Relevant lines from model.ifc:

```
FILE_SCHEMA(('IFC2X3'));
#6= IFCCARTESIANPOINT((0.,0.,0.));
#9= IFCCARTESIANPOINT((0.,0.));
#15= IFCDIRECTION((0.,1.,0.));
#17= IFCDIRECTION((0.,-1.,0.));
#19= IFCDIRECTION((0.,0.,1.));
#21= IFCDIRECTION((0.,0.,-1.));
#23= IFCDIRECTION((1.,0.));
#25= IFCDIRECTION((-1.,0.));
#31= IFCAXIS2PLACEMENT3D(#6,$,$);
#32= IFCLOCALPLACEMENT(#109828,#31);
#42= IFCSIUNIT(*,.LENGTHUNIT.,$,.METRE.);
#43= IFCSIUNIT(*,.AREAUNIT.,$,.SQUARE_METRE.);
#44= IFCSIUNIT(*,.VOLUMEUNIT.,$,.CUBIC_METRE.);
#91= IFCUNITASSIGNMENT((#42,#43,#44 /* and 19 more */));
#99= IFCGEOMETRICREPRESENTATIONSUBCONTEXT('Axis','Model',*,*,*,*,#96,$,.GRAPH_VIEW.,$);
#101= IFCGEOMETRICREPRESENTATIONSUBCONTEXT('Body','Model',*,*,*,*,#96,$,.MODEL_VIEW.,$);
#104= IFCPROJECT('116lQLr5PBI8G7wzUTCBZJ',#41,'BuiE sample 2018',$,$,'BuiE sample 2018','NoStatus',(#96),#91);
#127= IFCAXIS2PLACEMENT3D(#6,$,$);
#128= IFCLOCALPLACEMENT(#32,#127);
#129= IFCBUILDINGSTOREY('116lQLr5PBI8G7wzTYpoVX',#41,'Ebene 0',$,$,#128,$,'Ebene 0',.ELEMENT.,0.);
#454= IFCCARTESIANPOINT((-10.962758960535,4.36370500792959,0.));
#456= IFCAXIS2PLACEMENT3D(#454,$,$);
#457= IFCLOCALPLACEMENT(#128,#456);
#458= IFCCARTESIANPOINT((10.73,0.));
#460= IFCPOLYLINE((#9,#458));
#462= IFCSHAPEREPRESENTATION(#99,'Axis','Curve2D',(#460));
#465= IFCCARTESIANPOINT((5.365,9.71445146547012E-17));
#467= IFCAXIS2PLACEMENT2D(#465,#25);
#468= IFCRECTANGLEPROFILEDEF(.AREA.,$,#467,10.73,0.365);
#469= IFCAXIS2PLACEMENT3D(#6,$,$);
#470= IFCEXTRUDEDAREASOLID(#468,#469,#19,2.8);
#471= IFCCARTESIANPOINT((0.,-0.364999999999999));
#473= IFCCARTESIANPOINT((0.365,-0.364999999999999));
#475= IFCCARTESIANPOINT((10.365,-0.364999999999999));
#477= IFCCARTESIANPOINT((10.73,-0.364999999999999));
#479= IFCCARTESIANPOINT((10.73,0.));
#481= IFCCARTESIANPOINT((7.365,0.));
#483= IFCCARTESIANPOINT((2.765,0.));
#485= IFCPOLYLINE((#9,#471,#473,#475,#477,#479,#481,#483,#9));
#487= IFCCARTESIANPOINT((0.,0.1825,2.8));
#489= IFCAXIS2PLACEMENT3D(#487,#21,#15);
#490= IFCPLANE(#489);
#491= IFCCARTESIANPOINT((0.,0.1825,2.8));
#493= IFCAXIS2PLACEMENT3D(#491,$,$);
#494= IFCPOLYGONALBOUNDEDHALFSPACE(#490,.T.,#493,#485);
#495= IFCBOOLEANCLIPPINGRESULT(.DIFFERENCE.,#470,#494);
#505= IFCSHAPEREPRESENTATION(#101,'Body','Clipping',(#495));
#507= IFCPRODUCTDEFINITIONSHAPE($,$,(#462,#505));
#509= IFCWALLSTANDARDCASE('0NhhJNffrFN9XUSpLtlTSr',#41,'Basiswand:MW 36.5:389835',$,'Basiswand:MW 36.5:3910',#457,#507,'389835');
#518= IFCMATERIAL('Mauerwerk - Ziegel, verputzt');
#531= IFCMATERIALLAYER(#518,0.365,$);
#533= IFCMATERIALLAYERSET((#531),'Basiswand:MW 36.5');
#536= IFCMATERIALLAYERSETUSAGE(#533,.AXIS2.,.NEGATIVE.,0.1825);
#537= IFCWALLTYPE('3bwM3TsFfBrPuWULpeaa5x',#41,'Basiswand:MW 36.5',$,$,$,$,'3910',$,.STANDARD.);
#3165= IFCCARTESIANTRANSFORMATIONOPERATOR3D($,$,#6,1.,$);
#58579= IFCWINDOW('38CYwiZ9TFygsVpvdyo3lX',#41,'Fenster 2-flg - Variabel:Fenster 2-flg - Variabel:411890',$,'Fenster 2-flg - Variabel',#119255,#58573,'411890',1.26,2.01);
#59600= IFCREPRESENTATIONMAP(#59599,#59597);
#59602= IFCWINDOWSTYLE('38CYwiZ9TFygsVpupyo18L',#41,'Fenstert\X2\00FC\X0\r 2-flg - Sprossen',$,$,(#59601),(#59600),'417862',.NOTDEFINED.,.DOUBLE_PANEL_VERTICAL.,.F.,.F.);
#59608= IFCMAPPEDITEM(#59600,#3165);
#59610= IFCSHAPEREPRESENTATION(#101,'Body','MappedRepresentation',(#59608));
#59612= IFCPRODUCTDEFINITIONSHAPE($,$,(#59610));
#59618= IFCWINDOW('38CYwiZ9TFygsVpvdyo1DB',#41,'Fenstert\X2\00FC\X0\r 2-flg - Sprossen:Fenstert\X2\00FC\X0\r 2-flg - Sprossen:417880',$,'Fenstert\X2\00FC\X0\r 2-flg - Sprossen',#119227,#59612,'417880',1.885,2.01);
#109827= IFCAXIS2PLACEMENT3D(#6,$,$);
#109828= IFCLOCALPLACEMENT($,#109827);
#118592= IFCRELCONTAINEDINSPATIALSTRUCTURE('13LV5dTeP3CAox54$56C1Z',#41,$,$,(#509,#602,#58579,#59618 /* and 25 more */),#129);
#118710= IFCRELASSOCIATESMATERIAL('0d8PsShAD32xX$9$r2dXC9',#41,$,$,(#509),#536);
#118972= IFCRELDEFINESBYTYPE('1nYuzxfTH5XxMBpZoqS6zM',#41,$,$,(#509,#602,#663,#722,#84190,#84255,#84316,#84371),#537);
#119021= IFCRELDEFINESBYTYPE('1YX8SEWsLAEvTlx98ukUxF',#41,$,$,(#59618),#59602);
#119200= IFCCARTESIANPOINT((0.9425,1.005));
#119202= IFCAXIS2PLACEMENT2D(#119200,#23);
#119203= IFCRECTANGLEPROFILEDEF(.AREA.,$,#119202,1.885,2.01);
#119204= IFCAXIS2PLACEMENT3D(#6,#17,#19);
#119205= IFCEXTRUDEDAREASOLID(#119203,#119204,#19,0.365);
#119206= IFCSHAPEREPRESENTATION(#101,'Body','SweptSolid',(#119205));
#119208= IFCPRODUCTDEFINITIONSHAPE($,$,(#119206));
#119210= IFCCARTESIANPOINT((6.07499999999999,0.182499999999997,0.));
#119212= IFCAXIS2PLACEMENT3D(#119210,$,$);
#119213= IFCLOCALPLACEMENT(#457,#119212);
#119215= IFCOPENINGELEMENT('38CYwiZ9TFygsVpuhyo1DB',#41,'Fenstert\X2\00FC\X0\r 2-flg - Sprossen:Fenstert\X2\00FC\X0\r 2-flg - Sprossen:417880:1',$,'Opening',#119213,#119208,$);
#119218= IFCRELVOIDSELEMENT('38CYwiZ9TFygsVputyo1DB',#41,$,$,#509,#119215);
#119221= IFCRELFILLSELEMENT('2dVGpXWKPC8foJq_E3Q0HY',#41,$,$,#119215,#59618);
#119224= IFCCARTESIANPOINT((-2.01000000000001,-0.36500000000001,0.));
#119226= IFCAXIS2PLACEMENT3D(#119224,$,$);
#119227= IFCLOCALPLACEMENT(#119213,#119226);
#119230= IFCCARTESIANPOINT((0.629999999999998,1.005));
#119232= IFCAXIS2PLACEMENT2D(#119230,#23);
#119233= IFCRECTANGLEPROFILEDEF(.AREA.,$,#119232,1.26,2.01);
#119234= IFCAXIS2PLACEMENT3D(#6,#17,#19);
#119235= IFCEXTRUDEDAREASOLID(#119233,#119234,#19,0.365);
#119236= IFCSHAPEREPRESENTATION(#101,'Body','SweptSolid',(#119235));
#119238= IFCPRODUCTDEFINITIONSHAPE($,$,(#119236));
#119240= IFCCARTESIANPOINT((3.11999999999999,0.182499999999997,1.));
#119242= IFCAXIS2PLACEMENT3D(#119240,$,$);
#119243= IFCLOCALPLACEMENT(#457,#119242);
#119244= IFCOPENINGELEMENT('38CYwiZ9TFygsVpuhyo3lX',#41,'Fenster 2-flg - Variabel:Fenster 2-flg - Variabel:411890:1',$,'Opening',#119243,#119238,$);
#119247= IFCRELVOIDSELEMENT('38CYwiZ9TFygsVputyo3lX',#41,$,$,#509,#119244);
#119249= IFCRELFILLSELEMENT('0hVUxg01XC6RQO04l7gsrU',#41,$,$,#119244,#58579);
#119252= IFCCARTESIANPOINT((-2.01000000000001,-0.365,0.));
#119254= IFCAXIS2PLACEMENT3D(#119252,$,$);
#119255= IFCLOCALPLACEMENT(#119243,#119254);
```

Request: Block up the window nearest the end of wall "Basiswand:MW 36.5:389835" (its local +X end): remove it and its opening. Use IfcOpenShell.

```python
import ifcopenshell
import ifcopenshell.api.feature
import ifcopenshell.api.root
import ifcopenshell.geom
import ifcopenshell.util.shape

model = ifcopenshell.open("model.ifc")
settings = ifcopenshell.geom.settings()


def volume(element):
    """Net volume in cubic metres, openings subtracted."""
    shape = ifcopenshell.geom.create_shape(settings, element)
    return ifcopenshell.util.shape.get_volume(shape.geometry)


window = model.by_guid("38CYwiZ9TFygsVpvdyo1DB")
opening = window.FillsVoids[0].RelatingOpeningElement
wall = opening.VoidsElements[0].RelatingBuildingElement
before = volume(wall)

ifcopenshell.api.root.remove_product(model, product=window)
ifcopenshell.api.feature.remove_feature(model, feature=opening)

after = volume(wall)

print(f"wall volume {before:.3f} -> {after:.3f} m3")

model.write("model_rev.ifc")
```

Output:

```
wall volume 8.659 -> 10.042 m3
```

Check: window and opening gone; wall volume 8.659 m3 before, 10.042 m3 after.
